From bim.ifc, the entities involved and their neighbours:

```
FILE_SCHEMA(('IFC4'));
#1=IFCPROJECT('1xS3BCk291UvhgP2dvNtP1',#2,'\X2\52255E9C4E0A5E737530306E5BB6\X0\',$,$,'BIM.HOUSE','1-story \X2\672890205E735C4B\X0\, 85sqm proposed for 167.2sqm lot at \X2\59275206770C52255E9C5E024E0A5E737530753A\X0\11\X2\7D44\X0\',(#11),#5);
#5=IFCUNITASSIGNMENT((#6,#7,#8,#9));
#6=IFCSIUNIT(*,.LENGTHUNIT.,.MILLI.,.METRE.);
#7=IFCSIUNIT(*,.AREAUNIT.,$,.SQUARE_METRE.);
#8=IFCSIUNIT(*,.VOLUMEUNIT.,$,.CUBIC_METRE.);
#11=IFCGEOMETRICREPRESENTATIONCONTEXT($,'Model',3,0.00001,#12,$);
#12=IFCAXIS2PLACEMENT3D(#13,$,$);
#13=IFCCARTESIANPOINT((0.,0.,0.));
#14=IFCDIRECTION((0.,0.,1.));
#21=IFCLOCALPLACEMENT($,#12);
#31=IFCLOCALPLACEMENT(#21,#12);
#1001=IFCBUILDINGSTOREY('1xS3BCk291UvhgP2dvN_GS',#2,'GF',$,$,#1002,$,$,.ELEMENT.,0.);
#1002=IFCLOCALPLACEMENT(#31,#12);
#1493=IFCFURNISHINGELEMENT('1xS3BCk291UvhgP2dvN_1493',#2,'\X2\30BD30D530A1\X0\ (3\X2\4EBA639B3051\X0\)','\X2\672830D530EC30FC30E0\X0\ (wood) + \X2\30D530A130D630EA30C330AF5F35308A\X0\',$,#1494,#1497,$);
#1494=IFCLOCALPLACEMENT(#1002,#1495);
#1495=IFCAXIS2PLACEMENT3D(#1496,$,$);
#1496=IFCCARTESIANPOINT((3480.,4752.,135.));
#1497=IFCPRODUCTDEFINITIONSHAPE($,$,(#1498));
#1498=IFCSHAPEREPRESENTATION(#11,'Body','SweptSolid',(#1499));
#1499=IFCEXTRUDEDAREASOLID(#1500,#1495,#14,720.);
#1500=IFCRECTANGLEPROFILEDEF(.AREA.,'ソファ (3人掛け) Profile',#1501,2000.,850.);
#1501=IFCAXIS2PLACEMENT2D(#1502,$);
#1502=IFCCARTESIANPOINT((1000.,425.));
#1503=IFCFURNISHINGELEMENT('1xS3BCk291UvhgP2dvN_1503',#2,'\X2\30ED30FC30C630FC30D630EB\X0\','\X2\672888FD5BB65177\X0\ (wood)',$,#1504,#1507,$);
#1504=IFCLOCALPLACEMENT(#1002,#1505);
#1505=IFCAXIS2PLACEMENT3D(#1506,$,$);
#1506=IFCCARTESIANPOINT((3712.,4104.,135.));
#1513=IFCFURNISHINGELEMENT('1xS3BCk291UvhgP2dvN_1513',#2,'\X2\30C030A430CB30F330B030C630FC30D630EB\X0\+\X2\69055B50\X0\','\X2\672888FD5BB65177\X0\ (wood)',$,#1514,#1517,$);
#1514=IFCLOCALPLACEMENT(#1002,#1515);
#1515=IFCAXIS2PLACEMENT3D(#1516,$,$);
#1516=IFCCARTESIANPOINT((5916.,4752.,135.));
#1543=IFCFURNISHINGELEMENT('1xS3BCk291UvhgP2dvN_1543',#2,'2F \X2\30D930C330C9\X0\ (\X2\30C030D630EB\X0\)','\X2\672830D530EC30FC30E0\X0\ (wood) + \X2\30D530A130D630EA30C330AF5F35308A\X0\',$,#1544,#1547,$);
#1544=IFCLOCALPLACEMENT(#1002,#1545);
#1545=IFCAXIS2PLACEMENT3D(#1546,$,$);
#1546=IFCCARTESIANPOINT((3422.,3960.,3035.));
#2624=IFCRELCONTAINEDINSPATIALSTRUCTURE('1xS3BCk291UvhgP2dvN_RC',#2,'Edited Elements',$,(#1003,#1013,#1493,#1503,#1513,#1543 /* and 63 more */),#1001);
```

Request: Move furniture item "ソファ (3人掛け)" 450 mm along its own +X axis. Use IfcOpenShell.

```python
import ifcopenshell
import ifcopenshell.api.geometry
import ifcopenshell.util.placement
import ifcopenshell.util.unit

model = ifcopenshell.open("bim.ifc")
unit_scale = ifcopenshell.util.unit.calculate_unit_scale(model)

item = model.by_guid("1xS3BCk291UvhgP2dvN_1493")
matrix = ifcopenshell.util.placement.get_local_placement(item.ObjectPlacement)
matrix[:3, 3] += matrix[:3, 0] * 0.45 / unit_scale
ifcopenshell.api.geometry.edit_object_placement(model, product=item, matrix=matrix, is_si=False)

print(ifcopenshell.util.placement.get_local_placement(item.ObjectPlacement).round(3) + 0.0)

model.write("bim_rev.ifc")
```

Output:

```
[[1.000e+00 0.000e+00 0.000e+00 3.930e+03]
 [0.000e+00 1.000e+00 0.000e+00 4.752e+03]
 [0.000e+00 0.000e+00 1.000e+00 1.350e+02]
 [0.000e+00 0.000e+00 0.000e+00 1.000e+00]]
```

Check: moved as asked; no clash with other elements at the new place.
